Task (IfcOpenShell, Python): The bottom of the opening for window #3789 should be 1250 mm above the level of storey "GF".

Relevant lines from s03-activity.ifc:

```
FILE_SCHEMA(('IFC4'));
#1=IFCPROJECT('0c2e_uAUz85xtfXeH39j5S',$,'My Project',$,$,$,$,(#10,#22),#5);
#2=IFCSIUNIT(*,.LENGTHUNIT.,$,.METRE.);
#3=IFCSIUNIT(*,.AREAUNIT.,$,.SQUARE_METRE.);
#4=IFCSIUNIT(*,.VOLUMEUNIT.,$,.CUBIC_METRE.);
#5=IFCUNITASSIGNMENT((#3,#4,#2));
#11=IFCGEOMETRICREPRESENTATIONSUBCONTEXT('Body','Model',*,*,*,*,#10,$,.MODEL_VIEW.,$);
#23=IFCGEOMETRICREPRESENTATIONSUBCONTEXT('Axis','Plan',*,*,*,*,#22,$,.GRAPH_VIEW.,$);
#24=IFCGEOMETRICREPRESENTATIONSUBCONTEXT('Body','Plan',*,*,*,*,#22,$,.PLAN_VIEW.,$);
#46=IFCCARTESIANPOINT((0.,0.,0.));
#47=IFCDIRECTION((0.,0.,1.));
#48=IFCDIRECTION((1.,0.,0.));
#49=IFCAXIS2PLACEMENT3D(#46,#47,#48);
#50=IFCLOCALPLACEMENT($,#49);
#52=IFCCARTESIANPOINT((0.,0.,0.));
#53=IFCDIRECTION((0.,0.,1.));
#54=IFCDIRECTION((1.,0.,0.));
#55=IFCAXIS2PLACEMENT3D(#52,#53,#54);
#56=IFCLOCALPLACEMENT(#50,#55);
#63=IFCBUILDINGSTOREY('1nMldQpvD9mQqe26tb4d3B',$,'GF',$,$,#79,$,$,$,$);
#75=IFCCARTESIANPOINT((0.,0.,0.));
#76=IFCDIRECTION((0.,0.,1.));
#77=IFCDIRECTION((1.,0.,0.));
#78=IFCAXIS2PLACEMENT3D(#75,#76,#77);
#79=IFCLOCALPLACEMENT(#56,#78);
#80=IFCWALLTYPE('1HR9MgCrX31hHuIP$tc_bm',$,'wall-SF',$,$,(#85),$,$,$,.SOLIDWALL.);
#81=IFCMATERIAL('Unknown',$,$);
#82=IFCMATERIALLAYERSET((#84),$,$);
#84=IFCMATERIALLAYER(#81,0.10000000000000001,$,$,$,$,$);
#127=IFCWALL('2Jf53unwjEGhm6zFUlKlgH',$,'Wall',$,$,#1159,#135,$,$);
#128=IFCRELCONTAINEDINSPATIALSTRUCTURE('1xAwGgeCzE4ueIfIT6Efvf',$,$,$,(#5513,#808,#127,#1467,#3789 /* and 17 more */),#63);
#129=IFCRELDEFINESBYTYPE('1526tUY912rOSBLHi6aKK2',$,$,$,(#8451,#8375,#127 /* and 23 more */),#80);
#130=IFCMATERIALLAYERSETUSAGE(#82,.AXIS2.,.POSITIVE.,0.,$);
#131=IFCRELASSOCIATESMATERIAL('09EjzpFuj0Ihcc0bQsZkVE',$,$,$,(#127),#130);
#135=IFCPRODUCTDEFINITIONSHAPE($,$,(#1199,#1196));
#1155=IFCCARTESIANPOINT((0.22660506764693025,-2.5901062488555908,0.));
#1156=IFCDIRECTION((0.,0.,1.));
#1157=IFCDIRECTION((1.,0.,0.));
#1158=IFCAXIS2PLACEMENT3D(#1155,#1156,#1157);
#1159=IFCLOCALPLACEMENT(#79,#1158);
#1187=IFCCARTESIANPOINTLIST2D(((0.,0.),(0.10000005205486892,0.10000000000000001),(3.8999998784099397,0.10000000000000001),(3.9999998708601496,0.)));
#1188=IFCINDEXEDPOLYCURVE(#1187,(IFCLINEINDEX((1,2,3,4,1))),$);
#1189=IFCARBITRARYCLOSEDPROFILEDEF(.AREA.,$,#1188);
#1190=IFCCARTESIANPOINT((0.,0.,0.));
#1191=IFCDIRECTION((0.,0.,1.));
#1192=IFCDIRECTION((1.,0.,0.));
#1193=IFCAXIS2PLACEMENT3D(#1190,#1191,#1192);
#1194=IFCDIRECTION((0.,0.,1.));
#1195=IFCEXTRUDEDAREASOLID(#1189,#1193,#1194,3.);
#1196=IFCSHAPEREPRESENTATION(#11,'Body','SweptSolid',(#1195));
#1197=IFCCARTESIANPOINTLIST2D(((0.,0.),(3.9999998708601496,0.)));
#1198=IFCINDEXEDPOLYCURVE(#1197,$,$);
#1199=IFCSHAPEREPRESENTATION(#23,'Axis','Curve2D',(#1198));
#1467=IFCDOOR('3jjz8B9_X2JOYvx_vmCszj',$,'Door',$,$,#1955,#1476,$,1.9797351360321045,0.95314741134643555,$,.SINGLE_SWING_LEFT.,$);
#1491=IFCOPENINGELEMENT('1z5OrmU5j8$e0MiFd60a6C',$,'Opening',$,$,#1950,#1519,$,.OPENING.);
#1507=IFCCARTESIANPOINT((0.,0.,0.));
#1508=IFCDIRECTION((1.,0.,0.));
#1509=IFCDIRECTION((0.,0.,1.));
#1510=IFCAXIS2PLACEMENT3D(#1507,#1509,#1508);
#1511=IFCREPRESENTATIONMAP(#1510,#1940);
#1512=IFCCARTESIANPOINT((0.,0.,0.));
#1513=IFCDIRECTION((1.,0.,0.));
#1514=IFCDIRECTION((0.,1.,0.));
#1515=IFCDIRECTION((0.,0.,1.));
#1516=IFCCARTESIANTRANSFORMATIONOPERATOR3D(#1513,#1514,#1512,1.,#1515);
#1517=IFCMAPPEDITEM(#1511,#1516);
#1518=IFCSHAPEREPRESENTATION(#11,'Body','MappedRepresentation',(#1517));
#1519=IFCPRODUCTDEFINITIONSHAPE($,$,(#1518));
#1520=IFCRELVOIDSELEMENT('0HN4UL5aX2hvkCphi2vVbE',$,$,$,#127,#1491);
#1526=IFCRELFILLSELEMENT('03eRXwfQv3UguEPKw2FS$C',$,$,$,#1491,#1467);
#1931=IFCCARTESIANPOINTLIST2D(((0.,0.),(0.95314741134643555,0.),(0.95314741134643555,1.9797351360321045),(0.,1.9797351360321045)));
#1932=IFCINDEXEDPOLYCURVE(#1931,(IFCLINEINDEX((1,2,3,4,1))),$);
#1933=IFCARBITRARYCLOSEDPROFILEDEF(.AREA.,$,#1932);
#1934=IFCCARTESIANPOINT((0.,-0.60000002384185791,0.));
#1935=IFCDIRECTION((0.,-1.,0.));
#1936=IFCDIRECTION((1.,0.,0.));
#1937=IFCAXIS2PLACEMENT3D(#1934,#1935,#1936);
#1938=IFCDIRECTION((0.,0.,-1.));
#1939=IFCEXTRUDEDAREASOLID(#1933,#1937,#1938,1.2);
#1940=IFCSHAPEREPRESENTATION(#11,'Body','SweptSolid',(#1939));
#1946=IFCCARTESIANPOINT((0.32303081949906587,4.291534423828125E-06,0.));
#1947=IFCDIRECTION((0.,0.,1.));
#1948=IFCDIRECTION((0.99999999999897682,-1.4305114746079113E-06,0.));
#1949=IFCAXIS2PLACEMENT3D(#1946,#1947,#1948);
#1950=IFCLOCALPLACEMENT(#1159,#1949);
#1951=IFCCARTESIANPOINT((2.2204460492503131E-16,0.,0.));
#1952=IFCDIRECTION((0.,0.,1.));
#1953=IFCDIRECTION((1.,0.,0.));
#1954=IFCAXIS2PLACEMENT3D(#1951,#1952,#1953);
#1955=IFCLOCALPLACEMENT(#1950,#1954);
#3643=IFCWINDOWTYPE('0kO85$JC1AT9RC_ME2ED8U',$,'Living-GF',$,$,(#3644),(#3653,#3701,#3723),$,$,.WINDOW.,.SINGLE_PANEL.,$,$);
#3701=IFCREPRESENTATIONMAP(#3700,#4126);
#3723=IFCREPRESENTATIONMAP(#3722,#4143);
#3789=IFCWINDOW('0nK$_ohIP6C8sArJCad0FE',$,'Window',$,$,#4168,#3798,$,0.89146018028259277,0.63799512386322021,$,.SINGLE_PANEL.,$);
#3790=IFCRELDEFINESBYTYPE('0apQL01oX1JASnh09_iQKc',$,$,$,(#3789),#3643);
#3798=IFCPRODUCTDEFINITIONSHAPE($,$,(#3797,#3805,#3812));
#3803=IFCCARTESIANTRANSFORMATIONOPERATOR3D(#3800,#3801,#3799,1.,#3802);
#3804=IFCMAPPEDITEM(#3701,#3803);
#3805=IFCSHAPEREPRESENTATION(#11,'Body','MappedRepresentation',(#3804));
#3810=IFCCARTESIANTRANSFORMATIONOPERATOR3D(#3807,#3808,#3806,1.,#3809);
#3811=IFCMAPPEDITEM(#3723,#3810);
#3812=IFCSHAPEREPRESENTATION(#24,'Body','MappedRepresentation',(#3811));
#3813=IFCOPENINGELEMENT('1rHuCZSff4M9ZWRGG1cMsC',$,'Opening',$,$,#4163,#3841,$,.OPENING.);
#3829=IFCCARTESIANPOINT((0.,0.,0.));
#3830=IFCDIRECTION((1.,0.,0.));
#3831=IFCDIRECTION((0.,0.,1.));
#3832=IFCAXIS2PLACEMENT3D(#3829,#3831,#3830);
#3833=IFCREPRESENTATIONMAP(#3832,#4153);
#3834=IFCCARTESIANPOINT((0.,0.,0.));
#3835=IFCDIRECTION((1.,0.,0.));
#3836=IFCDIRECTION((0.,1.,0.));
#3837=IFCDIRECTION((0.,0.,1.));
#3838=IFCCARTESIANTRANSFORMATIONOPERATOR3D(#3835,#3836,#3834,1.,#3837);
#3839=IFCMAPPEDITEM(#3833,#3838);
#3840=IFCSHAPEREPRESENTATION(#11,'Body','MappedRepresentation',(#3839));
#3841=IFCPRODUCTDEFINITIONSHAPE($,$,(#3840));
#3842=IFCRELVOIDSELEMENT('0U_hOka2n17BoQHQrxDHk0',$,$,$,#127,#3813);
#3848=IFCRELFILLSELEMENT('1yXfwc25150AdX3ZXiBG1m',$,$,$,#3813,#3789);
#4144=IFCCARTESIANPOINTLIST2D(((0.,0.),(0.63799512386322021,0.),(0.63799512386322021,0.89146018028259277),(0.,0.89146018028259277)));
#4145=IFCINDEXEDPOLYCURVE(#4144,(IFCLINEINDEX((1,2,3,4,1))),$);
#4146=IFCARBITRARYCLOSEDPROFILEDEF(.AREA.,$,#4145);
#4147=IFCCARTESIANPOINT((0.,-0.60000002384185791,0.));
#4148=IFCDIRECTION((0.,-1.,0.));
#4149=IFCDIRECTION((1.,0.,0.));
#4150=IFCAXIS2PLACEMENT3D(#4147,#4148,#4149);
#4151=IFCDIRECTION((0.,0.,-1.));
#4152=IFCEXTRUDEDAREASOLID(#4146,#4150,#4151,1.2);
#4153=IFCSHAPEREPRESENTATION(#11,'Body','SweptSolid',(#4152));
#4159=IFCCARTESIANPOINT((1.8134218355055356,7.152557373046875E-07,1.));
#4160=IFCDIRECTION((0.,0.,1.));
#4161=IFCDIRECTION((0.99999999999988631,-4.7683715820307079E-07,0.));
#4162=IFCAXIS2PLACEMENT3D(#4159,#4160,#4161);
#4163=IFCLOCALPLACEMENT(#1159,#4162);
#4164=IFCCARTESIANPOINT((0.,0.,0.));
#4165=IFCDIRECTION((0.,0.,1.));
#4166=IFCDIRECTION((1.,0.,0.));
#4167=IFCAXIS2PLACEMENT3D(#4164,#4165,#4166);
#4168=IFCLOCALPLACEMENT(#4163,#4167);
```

```python
import numpy as np
import ifcopenshell
import ifcopenshell.api.geometry
import ifcopenshell.geom
import ifcopenshell.util.element
import ifcopenshell.util.placement
import ifcopenshell.util.shape
import ifcopenshell.util.unit

model = ifcopenshell.open("s03-activity.ifc")
unit_scale = ifcopenshell.util.unit.calculate_unit_scale(model)

window = model.by_guid("0nK$_ohIP6C8sArJCad0FE")
opening = window.FillsVoids[0].RelatingOpeningElement
storey = ifcopenshell.util.element.get_container(window, ifc_class="IfcBuildingStorey")
level = ifcopenshell.util.placement.get_local_placement(storey.ObjectPlacement)[2, 3]

# The opening's origin need not be at the sill, so measure its lowest point.
shape = ifcopenshell.geom.create_shape(ifcopenshell.geom.settings(), opening)
bottom = ifcopenshell.util.shape.get_shape_bottom_elevation(shape, shape.geometry) / unit_scale
dz = level + 1.25 / unit_scale - bottom

shift = np.array([0.0, 0.0, dz])
# The window is placed relative to its opening, so it follows when the opening moves.
matrix = ifcopenshell.util.placement.get_local_placement(opening.ObjectPlacement)
matrix[:3, 3] += shift
ifcopenshell.api.geometry.edit_object_placement(
    model, product=opening, matrix=matrix, is_si=False, should_transform_children=True
)

print(f"moved by {dz * unit_scale:+.3f} m")

model.write("s03-activity_rev.ifc")
```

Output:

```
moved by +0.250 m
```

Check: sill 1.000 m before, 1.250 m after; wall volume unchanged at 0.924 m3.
